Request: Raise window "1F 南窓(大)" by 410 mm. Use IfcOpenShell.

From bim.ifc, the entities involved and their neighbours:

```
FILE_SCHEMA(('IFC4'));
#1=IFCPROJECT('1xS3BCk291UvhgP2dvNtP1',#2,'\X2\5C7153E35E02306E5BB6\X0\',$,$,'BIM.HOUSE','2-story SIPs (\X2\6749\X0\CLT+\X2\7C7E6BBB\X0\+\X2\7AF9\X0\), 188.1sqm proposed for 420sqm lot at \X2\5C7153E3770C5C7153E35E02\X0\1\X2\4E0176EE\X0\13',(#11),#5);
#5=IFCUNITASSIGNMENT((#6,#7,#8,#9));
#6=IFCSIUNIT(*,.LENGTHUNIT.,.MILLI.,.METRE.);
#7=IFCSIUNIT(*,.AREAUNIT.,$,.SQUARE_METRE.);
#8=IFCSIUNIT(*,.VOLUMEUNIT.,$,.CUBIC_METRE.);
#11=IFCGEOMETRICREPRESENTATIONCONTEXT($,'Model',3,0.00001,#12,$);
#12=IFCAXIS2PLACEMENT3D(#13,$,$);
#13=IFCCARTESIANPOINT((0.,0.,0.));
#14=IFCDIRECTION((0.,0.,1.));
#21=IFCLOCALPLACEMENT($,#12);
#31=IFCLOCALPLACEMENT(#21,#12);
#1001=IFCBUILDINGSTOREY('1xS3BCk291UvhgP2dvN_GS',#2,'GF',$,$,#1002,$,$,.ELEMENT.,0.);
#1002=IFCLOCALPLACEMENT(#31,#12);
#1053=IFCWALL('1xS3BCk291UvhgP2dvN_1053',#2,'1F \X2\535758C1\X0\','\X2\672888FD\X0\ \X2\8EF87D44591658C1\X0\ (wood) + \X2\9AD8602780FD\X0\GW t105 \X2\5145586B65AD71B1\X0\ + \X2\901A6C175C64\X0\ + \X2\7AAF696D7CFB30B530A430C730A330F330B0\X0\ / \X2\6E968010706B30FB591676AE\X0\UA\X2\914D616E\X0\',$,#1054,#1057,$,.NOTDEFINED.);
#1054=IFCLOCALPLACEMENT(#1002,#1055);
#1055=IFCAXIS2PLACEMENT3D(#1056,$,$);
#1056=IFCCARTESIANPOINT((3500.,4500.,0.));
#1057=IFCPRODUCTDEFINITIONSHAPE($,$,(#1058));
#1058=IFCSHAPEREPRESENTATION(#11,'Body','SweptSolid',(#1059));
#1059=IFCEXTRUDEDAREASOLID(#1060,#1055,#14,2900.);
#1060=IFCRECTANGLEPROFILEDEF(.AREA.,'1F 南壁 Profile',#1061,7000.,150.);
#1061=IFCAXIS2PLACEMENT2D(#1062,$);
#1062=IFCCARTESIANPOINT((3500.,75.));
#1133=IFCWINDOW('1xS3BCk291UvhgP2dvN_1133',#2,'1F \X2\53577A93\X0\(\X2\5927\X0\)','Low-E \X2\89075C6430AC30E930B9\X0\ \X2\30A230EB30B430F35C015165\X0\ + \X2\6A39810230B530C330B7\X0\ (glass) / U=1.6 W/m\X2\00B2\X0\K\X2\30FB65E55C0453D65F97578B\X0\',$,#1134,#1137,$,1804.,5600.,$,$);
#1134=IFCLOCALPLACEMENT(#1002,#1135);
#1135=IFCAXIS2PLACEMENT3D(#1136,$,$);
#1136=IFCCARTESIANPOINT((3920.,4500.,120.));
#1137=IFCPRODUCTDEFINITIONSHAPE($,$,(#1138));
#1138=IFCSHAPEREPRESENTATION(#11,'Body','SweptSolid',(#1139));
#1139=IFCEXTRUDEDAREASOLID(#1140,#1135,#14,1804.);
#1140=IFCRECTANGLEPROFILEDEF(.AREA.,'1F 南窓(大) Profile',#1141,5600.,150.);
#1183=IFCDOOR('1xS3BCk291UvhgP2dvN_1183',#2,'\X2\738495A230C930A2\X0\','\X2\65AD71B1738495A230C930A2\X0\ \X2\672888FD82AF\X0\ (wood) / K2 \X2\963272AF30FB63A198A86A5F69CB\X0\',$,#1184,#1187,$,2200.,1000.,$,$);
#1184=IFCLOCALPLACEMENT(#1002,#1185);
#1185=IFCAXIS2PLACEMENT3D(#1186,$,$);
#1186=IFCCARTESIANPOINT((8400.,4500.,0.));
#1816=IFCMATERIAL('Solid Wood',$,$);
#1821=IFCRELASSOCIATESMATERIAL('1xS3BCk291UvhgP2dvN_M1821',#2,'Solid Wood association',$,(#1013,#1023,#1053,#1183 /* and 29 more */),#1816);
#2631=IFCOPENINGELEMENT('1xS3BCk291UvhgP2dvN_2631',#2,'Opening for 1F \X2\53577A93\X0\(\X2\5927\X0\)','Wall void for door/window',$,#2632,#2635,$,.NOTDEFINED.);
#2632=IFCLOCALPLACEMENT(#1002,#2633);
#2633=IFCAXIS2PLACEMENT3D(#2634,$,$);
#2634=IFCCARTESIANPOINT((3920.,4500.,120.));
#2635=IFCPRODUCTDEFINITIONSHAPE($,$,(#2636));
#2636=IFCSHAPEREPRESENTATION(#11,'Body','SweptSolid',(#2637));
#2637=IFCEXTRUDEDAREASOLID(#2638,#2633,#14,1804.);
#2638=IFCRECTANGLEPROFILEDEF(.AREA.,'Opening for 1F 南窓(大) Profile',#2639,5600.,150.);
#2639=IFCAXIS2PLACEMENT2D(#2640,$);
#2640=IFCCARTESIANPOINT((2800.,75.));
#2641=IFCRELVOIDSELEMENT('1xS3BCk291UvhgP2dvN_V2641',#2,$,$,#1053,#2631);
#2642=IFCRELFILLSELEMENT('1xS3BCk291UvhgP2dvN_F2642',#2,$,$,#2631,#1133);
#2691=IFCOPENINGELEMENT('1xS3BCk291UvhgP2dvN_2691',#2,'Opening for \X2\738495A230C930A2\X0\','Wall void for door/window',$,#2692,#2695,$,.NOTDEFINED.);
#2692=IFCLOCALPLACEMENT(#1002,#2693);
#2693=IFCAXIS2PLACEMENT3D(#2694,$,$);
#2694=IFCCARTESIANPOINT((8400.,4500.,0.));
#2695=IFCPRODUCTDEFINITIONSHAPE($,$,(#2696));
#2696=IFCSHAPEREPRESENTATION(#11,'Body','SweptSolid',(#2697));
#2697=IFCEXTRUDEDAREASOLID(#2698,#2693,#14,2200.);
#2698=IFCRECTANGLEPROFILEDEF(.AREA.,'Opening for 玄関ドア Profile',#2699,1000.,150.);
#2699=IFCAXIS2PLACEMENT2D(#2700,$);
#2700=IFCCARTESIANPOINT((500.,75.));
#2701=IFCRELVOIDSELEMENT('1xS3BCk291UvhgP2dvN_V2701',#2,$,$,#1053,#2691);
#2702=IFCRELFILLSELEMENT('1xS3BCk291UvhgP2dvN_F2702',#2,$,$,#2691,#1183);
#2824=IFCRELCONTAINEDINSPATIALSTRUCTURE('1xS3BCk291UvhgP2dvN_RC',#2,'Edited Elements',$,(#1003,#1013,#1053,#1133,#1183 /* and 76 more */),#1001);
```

```python
import numpy as np
import ifcopenshell
import ifcopenshell.api.geometry
import ifcopenshell.util.placement
import ifcopenshell.util.unit

model = ifcopenshell.open("bim.ifc")
unit_scale = ifcopenshell.util.unit.calculate_unit_scale(model)

window = model.by_id(1133)
opening = window.FillsVoids[0].RelatingOpeningElement
dz = 0.41 / unit_scale

shift = np.array([0.0, 0.0, dz])
# The window is not placed relative to its opening, so move both.
for product in (opening, window):
    matrix = ifcopenshell.util.placement.get_local_placement(product.ObjectPlacement)
    matrix[:3, 3] += shift
    ifcopenshell.api.geometry.edit_object_placement(model, product=product, matrix=matrix, is_si=False)

print(f"moved by {dz * unit_scale:+.3f} m")

model.write("bim_edited.ifc")
```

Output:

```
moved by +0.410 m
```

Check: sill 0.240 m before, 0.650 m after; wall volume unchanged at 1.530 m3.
